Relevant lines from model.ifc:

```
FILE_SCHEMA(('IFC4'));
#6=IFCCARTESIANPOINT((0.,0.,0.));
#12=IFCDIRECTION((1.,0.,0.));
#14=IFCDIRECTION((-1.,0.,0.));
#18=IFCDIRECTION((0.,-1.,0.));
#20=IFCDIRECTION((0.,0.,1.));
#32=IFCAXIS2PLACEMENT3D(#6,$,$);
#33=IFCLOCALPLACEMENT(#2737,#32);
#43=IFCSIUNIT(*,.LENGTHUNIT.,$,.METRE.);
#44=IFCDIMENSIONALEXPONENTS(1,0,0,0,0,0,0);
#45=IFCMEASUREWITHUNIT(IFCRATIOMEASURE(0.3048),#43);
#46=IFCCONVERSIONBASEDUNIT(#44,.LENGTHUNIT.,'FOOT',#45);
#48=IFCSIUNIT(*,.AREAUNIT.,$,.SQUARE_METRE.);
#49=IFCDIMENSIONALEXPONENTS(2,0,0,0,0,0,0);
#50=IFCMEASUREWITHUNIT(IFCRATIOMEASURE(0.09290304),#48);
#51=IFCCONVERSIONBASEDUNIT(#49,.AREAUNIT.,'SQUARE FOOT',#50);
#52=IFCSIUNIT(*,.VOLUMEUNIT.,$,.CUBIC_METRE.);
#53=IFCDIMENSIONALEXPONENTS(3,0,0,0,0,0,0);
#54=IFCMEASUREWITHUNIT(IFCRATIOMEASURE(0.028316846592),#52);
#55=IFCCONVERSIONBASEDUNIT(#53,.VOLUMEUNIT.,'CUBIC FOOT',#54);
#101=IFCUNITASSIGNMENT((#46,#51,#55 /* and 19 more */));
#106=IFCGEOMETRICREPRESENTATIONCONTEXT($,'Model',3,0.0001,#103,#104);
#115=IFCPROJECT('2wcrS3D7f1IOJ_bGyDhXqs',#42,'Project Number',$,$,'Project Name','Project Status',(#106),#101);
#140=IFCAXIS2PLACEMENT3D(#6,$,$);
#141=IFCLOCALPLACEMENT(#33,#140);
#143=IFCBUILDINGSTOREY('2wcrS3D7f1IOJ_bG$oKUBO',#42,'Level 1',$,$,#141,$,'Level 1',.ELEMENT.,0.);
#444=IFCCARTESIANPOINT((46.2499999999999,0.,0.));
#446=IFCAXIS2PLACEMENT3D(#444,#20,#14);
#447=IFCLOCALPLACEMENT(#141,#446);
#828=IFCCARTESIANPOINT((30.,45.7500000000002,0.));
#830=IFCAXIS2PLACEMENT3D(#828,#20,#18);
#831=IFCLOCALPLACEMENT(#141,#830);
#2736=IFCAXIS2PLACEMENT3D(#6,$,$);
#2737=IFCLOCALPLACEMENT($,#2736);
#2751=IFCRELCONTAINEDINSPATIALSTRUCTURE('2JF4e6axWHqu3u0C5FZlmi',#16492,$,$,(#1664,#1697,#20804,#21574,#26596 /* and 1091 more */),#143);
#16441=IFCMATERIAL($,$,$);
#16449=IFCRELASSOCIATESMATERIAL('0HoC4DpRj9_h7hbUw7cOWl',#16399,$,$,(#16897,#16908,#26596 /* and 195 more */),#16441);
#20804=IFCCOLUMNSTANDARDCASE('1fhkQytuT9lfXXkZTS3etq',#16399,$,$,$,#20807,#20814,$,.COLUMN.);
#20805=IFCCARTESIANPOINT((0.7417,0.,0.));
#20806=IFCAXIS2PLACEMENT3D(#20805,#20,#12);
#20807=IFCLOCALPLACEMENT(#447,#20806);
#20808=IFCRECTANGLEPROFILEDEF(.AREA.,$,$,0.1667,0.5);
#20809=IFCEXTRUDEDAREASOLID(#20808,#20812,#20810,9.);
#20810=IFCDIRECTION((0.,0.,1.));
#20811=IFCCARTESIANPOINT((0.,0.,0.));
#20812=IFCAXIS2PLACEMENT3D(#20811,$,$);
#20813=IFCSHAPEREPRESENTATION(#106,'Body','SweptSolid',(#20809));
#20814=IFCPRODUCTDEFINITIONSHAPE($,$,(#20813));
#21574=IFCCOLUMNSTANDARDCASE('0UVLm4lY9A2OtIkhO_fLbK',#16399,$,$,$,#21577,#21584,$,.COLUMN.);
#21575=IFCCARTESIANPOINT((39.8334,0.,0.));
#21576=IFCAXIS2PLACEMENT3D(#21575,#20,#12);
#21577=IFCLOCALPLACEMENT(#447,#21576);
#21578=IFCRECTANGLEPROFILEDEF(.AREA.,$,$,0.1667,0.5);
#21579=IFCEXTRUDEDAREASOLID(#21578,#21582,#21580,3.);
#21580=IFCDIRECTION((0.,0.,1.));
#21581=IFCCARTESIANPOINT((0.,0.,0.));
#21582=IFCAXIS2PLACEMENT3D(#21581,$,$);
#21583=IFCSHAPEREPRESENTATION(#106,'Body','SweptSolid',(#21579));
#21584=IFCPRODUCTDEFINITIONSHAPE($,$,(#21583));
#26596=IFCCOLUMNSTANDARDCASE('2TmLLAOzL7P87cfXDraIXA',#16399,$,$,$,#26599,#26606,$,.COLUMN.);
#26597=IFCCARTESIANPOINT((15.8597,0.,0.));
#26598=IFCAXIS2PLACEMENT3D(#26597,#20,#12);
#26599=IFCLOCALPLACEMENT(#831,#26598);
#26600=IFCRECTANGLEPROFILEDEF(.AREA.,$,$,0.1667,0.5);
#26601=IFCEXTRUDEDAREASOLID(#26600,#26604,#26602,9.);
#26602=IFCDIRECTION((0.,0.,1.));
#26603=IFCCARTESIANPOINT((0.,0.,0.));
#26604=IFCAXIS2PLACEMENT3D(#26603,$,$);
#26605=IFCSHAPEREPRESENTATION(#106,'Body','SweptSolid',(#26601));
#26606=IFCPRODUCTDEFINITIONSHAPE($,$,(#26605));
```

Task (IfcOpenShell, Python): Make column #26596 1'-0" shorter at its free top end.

```python
import ifcopenshell
import ifcopenshell.util.unit

model = ifcopenshell.open("model.ifc")
unit_scale = ifcopenshell.util.unit.calculate_unit_scale(model)

member = model.by_guid("2TmLLAOzL7P87cfXDraIXA")
change = -12 * 0.0254 / unit_scale

# The extrusion runs towards the end named, so only its depth changes.
body = next(r for r in member.Representation.Representations if r.RepresentationIdentifier == "Body")
solid = body.Items[0]
old_length = solid.Depth
solid.Depth += change

print(f"length {old_length:g} -> {solid.Depth:g}")

model.write("model_edited.ifc")
```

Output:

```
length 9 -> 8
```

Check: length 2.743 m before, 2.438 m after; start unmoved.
